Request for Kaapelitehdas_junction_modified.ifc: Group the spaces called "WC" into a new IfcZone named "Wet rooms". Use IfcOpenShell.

First a look at what the model holds.

```python
import ifcopenshell

model = ifcopenshell.open("Kaapelitehdas_junction_modified.ifc")
print(model.schema)
seen = {}
for space in model.by_type("IfcSpace"):
    seen[space.LongName] = seen.get(space.LongName, 0) + 1
for name, count in sorted(seen.items(), key=str):
    print(count, "x", name)
print("zones:", [z.Name for z in model.by_type("IfcZone")][:20])
```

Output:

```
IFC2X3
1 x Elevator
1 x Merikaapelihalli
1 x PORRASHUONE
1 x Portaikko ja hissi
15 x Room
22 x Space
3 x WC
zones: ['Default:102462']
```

```python
import ifcopenshell
import ifcopenshell.api.group
import ifcopenshell.api.root

model = ifcopenshell.open("Kaapelitehdas_junction_modified.ifc")

names = {"WC"}
spaces = [s for s in model.by_type("IfcSpace") if s.LongName in names]

zone = ifcopenshell.api.root.create_entity(model, ifc_class="IfcZone", name="Wet rooms")
ifcopenshell.api.group.assign_group(model, products=spaces, group=zone)
print(len(spaces), "spaces in", zone.Name)

model.write("Kaapelitehdas_junction_modified_v2.ifc")
```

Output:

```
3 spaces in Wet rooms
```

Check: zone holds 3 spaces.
